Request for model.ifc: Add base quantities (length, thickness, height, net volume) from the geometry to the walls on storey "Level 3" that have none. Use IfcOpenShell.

First a look at what the model holds.

```python
import ifcopenshell
import ifcopenshell.util.element
import ifcopenshell.util.unit

model = ifcopenshell.open("model.ifc")
print(model.schema)
for unit_type in ("LENGTHUNIT", "AREAUNIT", "VOLUMEUNIT"):
    print(unit_type, ifcopenshell.util.unit.calculate_unit_scale(model, unit_type))
storey = next(s for s in model.by_type("IfcBuildingStorey") if s.Name == "Level 3")
walls = [e for e in ifcopenshell.util.element.get_decomposition(storey) if e.is_a("IfcWall")]
for e in sorted(walls, key=lambda e: e.id()):
    print(e.id(), e.is_a(), e.Name, list(ifcopenshell.util.element.get_psets(e, qtos_only=True)), sep=" | ")
```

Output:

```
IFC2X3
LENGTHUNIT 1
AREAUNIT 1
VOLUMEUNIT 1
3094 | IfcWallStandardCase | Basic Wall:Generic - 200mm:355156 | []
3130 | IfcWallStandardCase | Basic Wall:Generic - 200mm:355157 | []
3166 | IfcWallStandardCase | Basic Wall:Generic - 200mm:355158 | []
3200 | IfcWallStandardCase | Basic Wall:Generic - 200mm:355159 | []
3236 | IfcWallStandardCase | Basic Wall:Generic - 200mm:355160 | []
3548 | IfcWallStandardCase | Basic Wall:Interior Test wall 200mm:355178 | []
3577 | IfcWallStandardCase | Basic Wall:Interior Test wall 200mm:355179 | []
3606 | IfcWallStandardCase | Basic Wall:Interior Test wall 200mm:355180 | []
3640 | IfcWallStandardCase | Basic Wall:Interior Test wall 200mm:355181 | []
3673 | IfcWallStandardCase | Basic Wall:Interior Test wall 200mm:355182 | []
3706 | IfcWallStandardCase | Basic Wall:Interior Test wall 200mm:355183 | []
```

```python
import ifcopenshell
import ifcopenshell.api.pset
import ifcopenshell.geom
import ifcopenshell.util.element
import ifcopenshell.util.shape
import ifcopenshell.util.unit

model = ifcopenshell.open("model.ifc")
unit_scale = ifcopenshell.util.unit.calculate_unit_scale(model)
volume_scale = ifcopenshell.util.unit.calculate_unit_scale(model, "VOLUMEUNIT")
settings = ifcopenshell.geom.settings()

storey = next(s for s in model.by_type("IfcBuildingStorey") if s.Name == "Level 3")
walls = [e for e in ifcopenshell.util.element.get_decomposition(storey) if e.is_a("IfcWall")]

for e in sorted(walls, key=lambda e: e.id()):
    if ifcopenshell.util.element.get_psets(e, qtos_only=True, should_inherit=False):
        continue
    # Geometry comes back in metres, in the element's own axes.
    shape = ifcopenshell.geom.create_shape(settings, e)
    values = {
        "Length": ifcopenshell.util.shape.get_x(shape.geometry) / unit_scale,
        "Width": ifcopenshell.util.shape.get_y(shape.geometry) / unit_scale,
        "Height": ifcopenshell.util.shape.get_z(shape.geometry) / unit_scale,
        "NetVolume": ifcopenshell.util.shape.get_volume(shape.geometry) / volume_scale,
    }
    qto = ifcopenshell.api.pset.add_qto(model, product=e, name="BaseQuantities")
    ifcopenshell.api.pset.edit_qto(model, qto=qto, properties=values)
    print(e.id(), {k: round(v, 3) for k, v in values.items()})

model.write("model_updated.ifc")
```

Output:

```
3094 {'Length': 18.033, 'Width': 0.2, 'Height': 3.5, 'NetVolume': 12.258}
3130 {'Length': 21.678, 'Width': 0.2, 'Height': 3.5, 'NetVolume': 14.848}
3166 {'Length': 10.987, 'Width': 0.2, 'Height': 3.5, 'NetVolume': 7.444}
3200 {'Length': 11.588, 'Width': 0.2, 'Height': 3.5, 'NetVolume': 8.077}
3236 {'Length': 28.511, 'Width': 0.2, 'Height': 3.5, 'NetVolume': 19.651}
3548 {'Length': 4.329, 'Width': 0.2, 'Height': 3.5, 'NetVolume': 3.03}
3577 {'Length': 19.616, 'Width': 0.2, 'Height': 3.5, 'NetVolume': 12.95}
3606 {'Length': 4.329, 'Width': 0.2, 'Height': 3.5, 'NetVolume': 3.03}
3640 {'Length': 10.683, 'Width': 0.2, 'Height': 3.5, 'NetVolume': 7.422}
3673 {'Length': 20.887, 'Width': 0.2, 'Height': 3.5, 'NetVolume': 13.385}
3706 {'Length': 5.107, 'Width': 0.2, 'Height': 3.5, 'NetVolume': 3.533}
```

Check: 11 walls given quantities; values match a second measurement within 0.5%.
